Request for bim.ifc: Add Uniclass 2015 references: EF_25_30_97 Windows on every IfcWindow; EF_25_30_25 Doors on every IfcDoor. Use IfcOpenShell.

First a look at what the model holds.

```python
import ifcopenshell

model = ifcopenshell.open("bim.ifc")
print(model.schema)
print("classifications:", [c.Name for c in model.by_type("IfcClassification")])
for ifc_class in ("IfcDoor", "IfcRoof", "IfcStair", "IfcWall", "IfcWindow"):
    print(ifc_class, len(model.by_type(ifc_class)))
```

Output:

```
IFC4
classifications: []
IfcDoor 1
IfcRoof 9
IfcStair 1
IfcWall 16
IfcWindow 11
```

```python
import ifcopenshell
import ifcopenshell.api.classification

model = ifcopenshell.open("bim.ifc")

system = ifcopenshell.api.classification.add_classification(model, classification="Uniclass 2015")

codes = {
    "IfcWindow": ("EF_25_30_97", "Windows"),
    "IfcDoor": ("EF_25_30_25", "Doors"),
}
for ifc_class, (code, name) in codes.items():
    products = model.by_type(ifc_class)
    ifcopenshell.api.classification.add_reference(
        model, products=products, classification=system, identification=code, name=name
    )
    print(code, len(products))

model.write("bim_edited.ifc")
```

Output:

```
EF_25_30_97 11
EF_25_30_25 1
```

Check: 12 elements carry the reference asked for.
